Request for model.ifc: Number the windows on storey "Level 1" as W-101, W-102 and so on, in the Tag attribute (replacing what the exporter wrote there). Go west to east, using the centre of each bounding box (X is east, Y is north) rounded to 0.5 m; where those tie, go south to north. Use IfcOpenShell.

First a look at what the model holds.

```python
import ifcopenshell
import ifcopenshell.util.element
import ifcopenshell.util.placement

model = ifcopenshell.open("model.ifc")
print(model.schema)
storey = next(s for s in model.by_type("IfcBuildingStorey") if s.Name == "Level 1")
windows = [e for e in ifcopenshell.util.element.get_decomposition(storey) if e.is_a("IfcWindow")]
for e in sorted(windows, key=lambda e: e.id()):
    origin = ifcopenshell.util.placement.get_local_placement(e.ObjectPlacement)[:3, 3]
    print(e.id(), e.Tag, e.Name, origin.round(2) + 0.0, sep=" | ")
```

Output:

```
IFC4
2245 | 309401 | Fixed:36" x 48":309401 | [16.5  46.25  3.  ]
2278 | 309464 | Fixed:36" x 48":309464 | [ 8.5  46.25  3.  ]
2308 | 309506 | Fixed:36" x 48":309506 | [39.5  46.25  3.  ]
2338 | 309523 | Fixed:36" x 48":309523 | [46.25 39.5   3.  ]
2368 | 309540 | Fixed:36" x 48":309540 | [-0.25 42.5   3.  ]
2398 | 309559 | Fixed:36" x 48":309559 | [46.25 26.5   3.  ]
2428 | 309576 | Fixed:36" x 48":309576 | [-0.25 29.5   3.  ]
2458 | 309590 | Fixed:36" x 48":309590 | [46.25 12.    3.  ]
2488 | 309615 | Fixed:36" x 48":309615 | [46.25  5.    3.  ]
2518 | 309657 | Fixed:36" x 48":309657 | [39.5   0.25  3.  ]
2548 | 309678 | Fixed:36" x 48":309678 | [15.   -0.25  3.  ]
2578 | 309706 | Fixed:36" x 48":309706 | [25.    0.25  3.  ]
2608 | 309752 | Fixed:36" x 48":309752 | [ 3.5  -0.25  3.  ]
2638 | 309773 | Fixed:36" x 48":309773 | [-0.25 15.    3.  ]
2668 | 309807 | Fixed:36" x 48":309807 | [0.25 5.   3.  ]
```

```python
import ifcopenshell
import ifcopenshell.geom
import ifcopenshell.util.element
import ifcopenshell.util.shape

model = ifcopenshell.open("model.ifc")
settings = ifcopenshell.geom.settings()
settings.set("use-world-coords", True)


def centre(element):
    shape = ifcopenshell.geom.create_shape(settings, element)
    return ifcopenshell.util.shape.get_bbox_centroid(shape.geometry)


storey = next(s for s in model.by_type("IfcBuildingStorey") if s.Name == "Level 1")
windows = [e for e in ifcopenshell.util.element.get_decomposition(storey) if e.is_a("IfcWindow")]

# Insertion points can sit at a corner or the storey origin, so sort by the geometry (in metres).
centres = {e: centre(e) for e in windows}
windows.sort(key=lambda e: (round(centres[e][0] / 0.5), centres[e][1]))

for i, e in enumerate(windows, start=1):
    number = f"W-1{i:02d}"
    e.Tag = number
    print(e.id(), number)

model.write("model-out.ifc")
```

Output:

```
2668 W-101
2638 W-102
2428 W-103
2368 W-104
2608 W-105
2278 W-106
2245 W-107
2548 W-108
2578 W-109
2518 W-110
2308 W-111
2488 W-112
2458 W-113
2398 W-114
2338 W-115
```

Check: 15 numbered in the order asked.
